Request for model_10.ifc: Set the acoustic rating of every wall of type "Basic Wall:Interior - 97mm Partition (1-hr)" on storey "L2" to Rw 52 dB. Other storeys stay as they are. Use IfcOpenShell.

First a look at what the model holds.

```python
import ifcopenshell
import ifcopenshell.util.element

model = ifcopenshell.open("model_10.ifc")
print(model.schema)
storey = next(s for s in model.by_type("IfcBuildingStorey") if s.Name == "L2")
walls = [e for e in ifcopenshell.util.element.get_decomposition(storey) if e.is_a("IfcWall")]
seen = {}
for e in walls:
    element_type = ifcopenshell.util.element.get_type(e)
    key = (element_type.Name if element_type != e and element_type else None, ifcopenshell.util.element.get_pset(e, "Pset_WallCommon", "AcousticRating"))
    seen[key] = seen.get(key, 0) + 1
for (name, value), count in sorted(seen.items(), key=str):
    print(count, "x", name, "|", value)
```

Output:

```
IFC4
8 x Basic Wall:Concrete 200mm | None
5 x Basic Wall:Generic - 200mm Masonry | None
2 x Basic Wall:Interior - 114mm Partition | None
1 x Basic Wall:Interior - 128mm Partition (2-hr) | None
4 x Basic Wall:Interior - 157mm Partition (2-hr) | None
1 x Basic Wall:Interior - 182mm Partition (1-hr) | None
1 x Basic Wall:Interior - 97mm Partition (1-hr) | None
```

```python
import ifcopenshell
import ifcopenshell.api.pset
import ifcopenshell.util.element

model = ifcopenshell.open("model_10.ifc")

storey = next(s for s in model.by_type("IfcBuildingStorey") if s.Name == "L2")
walls = [e for e in ifcopenshell.util.element.get_decomposition(storey) if e.is_a("IfcWall")]

count = 0
for e in walls:
    element_type = ifcopenshell.util.element.get_type(e)
    if element_type in (None, e) or element_type.Name != "Basic Wall:Interior - 97mm Partition (1-hr)":
        continue
    # add_pset returns the element's existing set when there is one.
    pset = ifcopenshell.api.pset.add_pset(model, product=e, name="Pset_WallCommon")
    ifcopenshell.api.pset.edit_pset(model, pset=pset, properties={"AcousticRating": "Rw 52 dB"})
    count += 1

print(count, "walls updated")

model.write("model_10_edited.ifc")
```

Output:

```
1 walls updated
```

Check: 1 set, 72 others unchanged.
